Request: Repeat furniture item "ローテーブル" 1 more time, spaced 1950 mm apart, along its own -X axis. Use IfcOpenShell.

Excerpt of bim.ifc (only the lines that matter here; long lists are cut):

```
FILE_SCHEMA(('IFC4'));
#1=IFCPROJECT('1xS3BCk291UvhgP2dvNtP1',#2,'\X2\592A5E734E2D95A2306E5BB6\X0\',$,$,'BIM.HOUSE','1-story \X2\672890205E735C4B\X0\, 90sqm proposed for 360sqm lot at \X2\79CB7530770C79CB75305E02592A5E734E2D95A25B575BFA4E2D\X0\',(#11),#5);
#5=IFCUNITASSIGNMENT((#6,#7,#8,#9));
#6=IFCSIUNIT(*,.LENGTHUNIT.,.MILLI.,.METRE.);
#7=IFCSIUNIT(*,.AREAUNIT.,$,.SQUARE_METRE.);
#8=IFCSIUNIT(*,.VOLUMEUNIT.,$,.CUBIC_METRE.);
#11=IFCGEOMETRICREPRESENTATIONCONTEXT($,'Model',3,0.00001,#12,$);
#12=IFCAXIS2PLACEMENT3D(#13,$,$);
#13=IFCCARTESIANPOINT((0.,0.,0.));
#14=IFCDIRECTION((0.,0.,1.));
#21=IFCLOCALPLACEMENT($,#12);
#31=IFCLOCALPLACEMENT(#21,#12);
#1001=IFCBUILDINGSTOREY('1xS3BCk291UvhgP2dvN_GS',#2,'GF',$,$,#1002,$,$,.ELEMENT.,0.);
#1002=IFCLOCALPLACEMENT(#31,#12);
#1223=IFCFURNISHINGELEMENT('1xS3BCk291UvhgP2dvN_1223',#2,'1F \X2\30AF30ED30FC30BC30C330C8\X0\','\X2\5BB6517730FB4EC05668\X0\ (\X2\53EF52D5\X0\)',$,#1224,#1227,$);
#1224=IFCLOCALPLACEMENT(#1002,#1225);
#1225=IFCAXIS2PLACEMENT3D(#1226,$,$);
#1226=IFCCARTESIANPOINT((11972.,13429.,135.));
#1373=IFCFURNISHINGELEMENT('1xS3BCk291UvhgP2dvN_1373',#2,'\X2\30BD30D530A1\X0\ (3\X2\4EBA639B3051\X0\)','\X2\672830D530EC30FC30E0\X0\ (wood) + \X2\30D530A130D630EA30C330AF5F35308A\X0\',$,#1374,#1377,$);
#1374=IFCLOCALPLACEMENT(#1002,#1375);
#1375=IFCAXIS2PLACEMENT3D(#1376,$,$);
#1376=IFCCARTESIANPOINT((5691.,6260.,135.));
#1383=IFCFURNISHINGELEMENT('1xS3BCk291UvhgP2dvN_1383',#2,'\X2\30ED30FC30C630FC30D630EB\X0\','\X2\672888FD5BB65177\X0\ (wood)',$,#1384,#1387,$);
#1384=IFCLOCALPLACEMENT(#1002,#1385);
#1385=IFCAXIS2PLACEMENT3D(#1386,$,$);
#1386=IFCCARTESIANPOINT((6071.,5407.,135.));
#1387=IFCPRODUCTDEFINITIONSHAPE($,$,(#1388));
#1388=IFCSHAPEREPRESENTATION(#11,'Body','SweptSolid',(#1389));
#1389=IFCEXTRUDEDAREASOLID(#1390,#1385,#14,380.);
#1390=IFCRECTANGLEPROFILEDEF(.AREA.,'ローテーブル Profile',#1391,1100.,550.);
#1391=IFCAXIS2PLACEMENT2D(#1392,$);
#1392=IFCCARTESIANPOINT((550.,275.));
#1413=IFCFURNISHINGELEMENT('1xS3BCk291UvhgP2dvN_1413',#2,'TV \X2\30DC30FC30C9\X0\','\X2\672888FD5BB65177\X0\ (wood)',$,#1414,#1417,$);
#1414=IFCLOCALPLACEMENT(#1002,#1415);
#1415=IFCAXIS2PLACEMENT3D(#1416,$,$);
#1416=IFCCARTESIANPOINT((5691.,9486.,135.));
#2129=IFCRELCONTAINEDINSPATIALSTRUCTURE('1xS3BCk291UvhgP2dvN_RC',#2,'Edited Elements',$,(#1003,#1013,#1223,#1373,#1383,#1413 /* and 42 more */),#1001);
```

```python
import ifcopenshell
import ifcopenshell.api.geometry
import ifcopenshell.api.root
import ifcopenshell.util.element
import ifcopenshell.util.placement

model = ifcopenshell.open("bim.ifc")


def reuse_history(source, copy):
    """copy_class also copies each property set's owner history, people and application; keep the originals."""
    for rel in copy.IsDefinedBy:
        if rel.is_a("IfcRelDefinesByProperties") and (history := rel.RelatingPropertyDefinition.OwnerHistory):
            rel.RelatingPropertyDefinition.OwnerHistory = source.OwnerHistory
            ifcopenshell.util.element.remove_deep2(model, history)


source = model.by_guid("1xS3BCk291UvhgP2dvN_1383")
base = ifcopenshell.util.placement.get_local_placement(source.ObjectPlacement)
step = -base[:3, 0] * 1950.0

for i in range(1, 2):
    copy = ifcopenshell.api.root.copy_class(model, product=source)
    copy.Representation = ifcopenshell.util.element.copy_deep(
        model, source.Representation, exclude=["IfcGeometricRepresentationContext", "IfcRepresentationMap"]
    )
    reuse_history(source, copy)
    matrix = base.copy()
    matrix[:3, 3] += i * step
    print("added at", matrix[:3, 3].round(3) + 0.0)
    ifcopenshell.api.geometry.edit_object_placement(model, product=copy, matrix=matrix, is_si=False)

model.write("bim_v2.ifc")
```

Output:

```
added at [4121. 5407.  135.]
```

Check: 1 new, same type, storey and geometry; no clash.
